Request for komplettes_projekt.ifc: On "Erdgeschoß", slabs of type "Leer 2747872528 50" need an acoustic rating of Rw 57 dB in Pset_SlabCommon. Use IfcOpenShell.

First a look at what the model holds.

```python
import ifcopenshell
import ifcopenshell.util.element

model = ifcopenshell.open("komplettes_projekt.ifc")
print(model.schema)
storey = next(s for s in model.by_type("IfcBuildingStorey") if s.Name == "Erdgeschoß")
slabs = [e for e in ifcopenshell.util.element.get_decomposition(storey) if e.is_a("IfcSlab")]
seen = {}
for e in slabs:
    element_type = ifcopenshell.util.element.get_type(e)
    key = (element_type.Name if element_type != e and element_type else None, ifcopenshell.util.element.get_pset(e, "Pset_SlabCommon", "AcousticRating"))
    seen[key] = seen.get(key, 0) + 1
for (name, value), count in sorted(seen.items(), key=str):
    print(count, "x", name, "|", value)
```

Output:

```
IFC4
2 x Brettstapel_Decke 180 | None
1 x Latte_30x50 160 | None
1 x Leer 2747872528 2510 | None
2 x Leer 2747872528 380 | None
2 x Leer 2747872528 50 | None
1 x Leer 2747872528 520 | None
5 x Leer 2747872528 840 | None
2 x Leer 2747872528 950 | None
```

```python
import ifcopenshell
import ifcopenshell.api.pset
import ifcopenshell.util.element

model = ifcopenshell.open("komplettes_projekt.ifc")

storey = next(s for s in model.by_type("IfcBuildingStorey") if s.Name == "Erdgeschoß")
slabs = [e for e in ifcopenshell.util.element.get_decomposition(storey) if e.is_a("IfcSlab")]

count = 0
for e in slabs:
    element_type = ifcopenshell.util.element.get_type(e)
    if element_type in (None, e) or element_type.Name != "Leer 2747872528 50":
        continue
    # add_pset returns the element's existing set when there is one.
    pset = ifcopenshell.api.pset.add_pset(model, product=e, name="Pset_SlabCommon")
    ifcopenshell.api.pset.edit_pset(model, pset=pset, properties={"AcousticRating": "Rw 57 dB"})
    count += 1

print(count, "slabs updated")

model.write("komplettes_projekt_updated.ifc")
```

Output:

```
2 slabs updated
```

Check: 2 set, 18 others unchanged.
